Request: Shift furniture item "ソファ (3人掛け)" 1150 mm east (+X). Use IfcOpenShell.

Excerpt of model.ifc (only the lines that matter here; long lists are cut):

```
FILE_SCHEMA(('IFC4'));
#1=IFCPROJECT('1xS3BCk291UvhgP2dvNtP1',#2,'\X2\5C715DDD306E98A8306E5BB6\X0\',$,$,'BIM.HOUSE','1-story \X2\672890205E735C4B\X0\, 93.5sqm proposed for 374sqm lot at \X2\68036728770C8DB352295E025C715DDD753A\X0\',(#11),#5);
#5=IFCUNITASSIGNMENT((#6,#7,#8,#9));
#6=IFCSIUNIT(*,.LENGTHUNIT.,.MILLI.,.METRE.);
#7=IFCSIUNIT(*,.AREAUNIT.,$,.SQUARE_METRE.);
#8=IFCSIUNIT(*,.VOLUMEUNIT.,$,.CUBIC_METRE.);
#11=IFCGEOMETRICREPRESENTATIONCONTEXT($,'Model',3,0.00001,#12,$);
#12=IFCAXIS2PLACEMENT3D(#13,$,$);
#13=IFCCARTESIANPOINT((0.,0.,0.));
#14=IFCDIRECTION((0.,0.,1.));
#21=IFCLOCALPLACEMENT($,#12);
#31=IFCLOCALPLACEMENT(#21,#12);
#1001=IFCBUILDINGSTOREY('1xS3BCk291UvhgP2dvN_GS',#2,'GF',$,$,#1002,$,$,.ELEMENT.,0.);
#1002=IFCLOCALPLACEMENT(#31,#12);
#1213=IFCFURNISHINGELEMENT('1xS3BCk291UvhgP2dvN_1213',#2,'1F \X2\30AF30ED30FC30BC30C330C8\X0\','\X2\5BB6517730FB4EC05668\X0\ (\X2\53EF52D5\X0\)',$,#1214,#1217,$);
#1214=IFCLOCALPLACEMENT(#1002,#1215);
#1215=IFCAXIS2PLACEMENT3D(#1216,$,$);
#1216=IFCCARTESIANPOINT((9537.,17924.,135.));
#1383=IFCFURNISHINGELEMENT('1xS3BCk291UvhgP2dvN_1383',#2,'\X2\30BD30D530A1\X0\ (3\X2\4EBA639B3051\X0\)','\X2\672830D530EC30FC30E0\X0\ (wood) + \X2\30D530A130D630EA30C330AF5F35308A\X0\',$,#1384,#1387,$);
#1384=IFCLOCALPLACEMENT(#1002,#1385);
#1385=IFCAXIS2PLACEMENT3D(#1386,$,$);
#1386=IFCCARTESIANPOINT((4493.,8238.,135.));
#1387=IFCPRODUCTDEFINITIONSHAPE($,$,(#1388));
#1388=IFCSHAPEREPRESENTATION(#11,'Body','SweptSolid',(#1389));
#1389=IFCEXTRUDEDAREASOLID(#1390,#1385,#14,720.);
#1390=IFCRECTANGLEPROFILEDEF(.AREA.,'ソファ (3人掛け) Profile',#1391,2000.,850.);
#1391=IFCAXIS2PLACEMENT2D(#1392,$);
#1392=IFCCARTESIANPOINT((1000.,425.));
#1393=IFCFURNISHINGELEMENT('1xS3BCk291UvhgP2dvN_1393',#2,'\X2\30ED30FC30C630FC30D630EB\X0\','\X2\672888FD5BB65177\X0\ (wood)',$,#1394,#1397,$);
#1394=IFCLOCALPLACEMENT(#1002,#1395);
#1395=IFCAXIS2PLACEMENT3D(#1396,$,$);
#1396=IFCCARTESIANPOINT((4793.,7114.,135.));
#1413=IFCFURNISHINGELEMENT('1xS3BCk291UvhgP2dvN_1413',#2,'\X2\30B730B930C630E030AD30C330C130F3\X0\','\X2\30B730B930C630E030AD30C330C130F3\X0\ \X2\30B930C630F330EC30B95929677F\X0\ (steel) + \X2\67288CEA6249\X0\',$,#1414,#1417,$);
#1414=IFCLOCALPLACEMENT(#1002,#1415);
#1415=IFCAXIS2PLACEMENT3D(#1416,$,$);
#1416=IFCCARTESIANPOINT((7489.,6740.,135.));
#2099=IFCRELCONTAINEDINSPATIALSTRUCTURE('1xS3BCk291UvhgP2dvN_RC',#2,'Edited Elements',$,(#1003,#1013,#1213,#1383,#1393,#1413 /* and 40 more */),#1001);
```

```python
import ifcopenshell
import ifcopenshell.api.geometry
import ifcopenshell.util.placement

model = ifcopenshell.open("model.ifc")

item = model.by_id(1383)
matrix = ifcopenshell.util.placement.get_local_placement(item.ObjectPlacement)
matrix[0, 3] += 1150.0
ifcopenshell.api.geometry.edit_object_placement(model, product=item, matrix=matrix, is_si=False)

print(ifcopenshell.util.placement.get_local_placement(item.ObjectPlacement).round(3) + 0.0)

model.write("model-out.ifc")
```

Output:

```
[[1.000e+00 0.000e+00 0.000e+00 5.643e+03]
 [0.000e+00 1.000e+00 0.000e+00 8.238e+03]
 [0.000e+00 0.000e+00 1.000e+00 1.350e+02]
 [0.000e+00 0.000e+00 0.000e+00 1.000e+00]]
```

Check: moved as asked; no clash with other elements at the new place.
